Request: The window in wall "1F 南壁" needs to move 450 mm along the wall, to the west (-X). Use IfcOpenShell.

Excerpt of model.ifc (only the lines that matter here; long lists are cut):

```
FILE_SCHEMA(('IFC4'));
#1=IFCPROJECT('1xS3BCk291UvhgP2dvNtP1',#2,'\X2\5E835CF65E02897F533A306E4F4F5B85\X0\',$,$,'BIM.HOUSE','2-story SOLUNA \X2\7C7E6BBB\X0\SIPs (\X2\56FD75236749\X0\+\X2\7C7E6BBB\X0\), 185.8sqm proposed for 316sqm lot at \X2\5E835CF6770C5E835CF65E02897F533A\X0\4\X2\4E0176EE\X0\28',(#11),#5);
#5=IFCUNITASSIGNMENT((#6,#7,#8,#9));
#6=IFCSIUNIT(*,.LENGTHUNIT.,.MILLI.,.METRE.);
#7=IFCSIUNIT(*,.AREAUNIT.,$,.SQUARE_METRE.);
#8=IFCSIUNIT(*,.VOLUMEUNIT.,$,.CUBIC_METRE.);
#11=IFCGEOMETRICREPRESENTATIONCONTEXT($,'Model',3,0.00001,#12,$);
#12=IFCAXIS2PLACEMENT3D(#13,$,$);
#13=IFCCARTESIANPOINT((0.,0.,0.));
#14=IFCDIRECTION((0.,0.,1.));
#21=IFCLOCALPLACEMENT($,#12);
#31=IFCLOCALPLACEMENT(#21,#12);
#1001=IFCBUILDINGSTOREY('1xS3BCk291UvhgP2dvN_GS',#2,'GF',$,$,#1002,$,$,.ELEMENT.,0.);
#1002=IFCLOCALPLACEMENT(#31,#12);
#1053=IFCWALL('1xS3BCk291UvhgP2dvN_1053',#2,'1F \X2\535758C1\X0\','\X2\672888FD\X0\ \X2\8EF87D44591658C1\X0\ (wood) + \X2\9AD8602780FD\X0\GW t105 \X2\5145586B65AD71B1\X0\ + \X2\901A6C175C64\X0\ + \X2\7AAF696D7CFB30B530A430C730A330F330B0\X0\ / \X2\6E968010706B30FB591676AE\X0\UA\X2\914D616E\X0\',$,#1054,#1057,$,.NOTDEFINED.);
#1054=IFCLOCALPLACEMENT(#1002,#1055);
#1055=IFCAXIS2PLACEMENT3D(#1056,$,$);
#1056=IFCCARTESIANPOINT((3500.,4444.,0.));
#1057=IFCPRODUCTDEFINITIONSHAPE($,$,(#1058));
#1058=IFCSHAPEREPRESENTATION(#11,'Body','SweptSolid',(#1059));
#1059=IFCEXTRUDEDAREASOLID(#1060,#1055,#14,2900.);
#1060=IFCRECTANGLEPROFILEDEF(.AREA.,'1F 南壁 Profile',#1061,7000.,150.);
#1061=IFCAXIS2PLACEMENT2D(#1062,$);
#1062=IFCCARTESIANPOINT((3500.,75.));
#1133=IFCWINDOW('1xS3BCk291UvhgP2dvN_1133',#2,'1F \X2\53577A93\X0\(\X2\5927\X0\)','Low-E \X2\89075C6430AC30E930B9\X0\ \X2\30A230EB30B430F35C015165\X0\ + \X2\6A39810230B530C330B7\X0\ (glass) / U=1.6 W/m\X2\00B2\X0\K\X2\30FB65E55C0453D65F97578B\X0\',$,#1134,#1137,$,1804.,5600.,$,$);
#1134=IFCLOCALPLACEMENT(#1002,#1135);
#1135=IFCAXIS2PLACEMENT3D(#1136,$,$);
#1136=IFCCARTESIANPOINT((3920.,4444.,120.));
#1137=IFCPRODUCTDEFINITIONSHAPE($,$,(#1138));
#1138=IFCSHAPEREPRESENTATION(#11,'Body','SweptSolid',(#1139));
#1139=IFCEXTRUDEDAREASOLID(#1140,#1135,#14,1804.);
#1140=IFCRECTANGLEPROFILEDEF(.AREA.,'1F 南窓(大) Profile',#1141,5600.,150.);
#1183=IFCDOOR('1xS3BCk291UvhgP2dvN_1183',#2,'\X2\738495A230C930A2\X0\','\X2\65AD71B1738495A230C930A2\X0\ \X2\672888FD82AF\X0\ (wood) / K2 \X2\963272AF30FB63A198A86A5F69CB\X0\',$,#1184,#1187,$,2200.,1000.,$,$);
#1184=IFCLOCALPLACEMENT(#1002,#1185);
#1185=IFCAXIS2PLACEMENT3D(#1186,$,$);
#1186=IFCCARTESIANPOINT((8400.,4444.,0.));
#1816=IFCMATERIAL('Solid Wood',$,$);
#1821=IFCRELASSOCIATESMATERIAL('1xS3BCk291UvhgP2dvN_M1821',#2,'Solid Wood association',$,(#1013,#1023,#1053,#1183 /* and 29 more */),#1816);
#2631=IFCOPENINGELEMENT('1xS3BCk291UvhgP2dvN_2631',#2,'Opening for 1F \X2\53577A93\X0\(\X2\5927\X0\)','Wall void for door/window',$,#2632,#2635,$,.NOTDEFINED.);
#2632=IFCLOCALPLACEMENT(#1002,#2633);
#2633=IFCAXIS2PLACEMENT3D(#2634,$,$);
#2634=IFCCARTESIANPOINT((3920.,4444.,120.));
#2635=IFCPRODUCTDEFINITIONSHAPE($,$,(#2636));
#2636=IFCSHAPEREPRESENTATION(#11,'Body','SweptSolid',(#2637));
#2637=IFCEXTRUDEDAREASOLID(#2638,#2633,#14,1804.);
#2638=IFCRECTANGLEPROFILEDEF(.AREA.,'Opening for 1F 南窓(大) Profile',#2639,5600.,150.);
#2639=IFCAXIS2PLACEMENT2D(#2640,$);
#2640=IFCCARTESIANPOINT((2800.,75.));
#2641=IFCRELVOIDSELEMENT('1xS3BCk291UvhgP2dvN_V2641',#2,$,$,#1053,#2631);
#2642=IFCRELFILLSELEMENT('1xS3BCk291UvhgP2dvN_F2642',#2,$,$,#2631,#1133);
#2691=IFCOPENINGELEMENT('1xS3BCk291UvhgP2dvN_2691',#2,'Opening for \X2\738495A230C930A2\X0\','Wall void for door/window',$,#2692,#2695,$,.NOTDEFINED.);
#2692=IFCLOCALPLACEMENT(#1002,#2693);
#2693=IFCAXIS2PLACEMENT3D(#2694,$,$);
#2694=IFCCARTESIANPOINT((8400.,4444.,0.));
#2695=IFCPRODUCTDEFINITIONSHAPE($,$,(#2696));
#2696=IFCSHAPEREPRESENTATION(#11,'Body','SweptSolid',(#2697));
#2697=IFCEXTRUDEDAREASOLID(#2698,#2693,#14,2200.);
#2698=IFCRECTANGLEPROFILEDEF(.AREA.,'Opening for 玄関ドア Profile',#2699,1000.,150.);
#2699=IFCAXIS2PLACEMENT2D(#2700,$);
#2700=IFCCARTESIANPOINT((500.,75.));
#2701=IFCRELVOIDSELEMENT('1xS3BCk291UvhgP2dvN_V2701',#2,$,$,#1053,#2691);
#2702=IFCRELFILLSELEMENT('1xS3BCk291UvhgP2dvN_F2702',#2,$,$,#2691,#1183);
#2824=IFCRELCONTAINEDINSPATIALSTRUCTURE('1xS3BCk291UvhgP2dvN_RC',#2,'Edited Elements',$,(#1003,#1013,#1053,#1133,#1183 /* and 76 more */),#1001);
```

```python
import ifcopenshell
import ifcopenshell.api.geometry
import ifcopenshell.util.placement
import ifcopenshell.util.unit

model = ifcopenshell.open("model.ifc")
unit_scale = ifcopenshell.util.unit.calculate_unit_scale(model)

window = model.by_guid("1xS3BCk291UvhgP2dvN_1133")
opening = window.FillsVoids[0].RelatingOpeningElement
wall = opening.VoidsElements[0].RelatingBuildingElement

wall_matrix = ifcopenshell.util.placement.get_local_placement(wall.ObjectPlacement)
shift = wall_matrix[:3, 0] * -0.45 / unit_scale
before = ifcopenshell.util.placement.get_local_placement(window.ObjectPlacement)[:3, 3].copy()

# The window is not placed relative to its opening, so move both.
for product in (opening, window):
    matrix = ifcopenshell.util.placement.get_local_placement(product.ObjectPlacement)
    matrix[:3, 3] += shift
    ifcopenshell.api.geometry.edit_object_placement(model, product=product, matrix=matrix, is_si=False)

after = ifcopenshell.util.placement.get_local_placement(window.ObjectPlacement)[:3, 3]
print("window moved by", (after - before).round(3) + 0.0)

model.write("model_updated.ifc")
```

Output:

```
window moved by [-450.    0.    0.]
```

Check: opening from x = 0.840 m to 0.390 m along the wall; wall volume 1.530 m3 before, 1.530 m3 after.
